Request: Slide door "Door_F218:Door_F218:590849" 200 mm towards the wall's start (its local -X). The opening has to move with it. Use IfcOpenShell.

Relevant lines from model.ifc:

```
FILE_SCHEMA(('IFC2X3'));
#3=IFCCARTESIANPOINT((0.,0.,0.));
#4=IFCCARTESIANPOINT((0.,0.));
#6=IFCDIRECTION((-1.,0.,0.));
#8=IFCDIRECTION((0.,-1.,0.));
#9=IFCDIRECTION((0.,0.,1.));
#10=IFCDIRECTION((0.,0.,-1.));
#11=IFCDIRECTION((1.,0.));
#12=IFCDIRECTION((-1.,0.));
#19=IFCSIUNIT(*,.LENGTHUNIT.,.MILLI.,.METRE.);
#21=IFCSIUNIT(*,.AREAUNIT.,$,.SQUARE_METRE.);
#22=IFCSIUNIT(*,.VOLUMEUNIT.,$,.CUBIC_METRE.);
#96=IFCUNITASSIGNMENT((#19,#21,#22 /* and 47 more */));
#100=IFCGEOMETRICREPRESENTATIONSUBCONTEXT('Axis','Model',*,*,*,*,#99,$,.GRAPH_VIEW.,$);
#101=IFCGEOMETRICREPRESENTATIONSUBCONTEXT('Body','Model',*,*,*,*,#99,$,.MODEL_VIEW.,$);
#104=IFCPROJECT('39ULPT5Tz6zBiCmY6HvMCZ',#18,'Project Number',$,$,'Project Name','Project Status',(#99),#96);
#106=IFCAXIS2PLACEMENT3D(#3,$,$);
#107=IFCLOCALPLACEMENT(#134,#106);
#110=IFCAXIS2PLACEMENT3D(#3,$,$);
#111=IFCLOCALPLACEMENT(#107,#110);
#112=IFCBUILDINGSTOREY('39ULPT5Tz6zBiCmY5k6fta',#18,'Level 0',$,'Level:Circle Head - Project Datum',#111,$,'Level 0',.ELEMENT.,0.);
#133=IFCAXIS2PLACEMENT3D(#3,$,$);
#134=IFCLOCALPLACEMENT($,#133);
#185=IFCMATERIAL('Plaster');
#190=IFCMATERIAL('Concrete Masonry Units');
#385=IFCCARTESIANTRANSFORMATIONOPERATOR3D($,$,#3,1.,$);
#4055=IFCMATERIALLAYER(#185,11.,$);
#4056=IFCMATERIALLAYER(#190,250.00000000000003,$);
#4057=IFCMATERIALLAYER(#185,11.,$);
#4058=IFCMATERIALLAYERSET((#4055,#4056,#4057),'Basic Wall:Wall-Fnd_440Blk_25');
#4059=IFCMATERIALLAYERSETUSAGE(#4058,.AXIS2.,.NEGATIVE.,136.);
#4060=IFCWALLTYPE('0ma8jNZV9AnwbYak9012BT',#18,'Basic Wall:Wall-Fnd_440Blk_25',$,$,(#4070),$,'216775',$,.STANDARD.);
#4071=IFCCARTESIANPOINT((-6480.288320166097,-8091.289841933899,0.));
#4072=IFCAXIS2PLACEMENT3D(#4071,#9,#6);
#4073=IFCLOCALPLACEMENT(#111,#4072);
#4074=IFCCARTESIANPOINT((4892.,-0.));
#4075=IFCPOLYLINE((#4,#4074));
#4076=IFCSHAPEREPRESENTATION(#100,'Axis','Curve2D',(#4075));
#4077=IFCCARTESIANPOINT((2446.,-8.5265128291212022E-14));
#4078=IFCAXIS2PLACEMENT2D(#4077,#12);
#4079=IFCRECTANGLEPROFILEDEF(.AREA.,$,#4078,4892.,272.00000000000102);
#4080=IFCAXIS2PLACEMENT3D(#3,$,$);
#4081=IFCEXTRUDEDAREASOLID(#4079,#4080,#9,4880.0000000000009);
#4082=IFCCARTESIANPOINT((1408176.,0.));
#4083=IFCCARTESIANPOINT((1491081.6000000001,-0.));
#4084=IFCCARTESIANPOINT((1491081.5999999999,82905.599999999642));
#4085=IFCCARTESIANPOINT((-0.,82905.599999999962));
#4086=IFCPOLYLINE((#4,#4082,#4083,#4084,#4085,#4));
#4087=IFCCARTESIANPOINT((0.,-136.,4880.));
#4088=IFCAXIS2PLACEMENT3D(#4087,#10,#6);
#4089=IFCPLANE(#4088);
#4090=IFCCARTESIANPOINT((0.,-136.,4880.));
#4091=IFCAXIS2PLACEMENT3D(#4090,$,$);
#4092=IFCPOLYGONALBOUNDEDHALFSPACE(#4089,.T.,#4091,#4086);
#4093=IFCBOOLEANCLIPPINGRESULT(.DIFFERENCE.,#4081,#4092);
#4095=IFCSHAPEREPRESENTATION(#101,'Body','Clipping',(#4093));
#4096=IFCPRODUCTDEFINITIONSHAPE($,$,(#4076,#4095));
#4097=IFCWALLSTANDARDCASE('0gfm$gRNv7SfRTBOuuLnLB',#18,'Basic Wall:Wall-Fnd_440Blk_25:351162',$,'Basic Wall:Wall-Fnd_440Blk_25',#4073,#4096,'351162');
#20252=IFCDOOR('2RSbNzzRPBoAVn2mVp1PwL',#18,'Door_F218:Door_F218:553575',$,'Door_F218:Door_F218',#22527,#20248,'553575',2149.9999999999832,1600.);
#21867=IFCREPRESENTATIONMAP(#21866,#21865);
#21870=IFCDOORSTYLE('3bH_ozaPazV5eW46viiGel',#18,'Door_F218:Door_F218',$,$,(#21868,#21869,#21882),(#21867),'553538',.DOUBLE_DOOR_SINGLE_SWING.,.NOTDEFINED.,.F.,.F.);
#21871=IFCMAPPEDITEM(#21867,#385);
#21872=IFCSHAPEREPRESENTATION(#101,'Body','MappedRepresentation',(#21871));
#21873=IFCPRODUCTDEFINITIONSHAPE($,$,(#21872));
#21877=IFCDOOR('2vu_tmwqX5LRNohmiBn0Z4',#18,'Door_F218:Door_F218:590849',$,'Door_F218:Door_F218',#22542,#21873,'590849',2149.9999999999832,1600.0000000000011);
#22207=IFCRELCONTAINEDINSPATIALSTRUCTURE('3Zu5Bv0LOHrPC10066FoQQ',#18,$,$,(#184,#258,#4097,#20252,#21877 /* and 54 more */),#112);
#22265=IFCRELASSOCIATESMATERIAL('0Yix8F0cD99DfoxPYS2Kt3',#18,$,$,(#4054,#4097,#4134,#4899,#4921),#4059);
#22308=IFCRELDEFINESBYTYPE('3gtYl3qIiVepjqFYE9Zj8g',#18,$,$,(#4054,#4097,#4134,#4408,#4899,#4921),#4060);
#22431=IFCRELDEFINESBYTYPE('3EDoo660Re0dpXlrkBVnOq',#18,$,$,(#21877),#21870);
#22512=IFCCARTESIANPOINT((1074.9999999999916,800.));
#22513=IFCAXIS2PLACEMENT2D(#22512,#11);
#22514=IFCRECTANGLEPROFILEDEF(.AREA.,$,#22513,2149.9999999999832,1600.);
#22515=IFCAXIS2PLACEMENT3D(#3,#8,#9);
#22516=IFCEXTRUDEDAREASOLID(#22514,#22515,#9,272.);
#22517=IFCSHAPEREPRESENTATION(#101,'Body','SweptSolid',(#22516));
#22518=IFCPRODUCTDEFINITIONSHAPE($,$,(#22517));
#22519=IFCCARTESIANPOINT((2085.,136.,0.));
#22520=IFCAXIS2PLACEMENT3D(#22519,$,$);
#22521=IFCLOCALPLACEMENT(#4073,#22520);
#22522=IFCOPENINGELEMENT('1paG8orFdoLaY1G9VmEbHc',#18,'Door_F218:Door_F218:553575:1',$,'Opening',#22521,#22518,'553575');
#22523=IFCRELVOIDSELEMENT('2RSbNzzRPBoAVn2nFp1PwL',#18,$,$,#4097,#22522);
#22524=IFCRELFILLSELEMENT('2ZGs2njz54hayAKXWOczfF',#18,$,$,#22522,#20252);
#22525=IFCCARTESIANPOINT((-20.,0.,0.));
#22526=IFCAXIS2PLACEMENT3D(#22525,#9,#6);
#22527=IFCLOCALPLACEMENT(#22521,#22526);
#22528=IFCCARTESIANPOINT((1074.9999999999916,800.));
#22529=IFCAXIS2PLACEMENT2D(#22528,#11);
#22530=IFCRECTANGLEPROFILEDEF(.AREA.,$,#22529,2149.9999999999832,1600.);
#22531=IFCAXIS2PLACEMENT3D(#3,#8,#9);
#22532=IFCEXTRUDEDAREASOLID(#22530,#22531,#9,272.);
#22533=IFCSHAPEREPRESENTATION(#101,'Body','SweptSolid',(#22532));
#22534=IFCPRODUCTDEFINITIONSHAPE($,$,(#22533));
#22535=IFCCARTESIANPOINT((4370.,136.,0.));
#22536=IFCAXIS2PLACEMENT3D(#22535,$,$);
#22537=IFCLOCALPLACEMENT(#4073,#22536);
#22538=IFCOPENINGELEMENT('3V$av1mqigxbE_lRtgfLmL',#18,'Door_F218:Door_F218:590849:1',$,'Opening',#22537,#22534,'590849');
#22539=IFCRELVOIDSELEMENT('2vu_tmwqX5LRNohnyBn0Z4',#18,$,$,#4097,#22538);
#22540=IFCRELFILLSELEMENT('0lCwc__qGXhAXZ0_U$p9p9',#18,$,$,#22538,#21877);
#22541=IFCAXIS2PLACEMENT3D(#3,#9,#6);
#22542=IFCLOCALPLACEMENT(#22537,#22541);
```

```python
import ifcopenshell
import ifcopenshell.api.geometry
import ifcopenshell.util.placement

model = ifcopenshell.open("model.ifc")

door = model.by_id(21877)
opening = door.FillsVoids[0].RelatingOpeningElement
wall = opening.VoidsElements[0].RelatingBuildingElement

wall_matrix = ifcopenshell.util.placement.get_local_placement(wall.ObjectPlacement)
shift = wall_matrix[:3, 0] * -200.0
before = ifcopenshell.util.placement.get_local_placement(door.ObjectPlacement)[:3, 3].copy()

# The door is placed relative to its opening, so it follows when the opening moves.
matrix = ifcopenshell.util.placement.get_local_placement(opening.ObjectPlacement)
matrix[:3, 3] += shift
ifcopenshell.api.geometry.edit_object_placement(
    model, product=opening, matrix=matrix, is_si=False, should_transform_children=True
)

after = ifcopenshell.util.placement.get_local_placement(door.ObjectPlacement)[:3, 3]
print("door moved by", (after - before).round(3) + 0.0)

model.write("model_edited.ifc")
```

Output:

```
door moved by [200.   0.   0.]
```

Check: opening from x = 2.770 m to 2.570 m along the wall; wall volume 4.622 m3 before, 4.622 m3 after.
